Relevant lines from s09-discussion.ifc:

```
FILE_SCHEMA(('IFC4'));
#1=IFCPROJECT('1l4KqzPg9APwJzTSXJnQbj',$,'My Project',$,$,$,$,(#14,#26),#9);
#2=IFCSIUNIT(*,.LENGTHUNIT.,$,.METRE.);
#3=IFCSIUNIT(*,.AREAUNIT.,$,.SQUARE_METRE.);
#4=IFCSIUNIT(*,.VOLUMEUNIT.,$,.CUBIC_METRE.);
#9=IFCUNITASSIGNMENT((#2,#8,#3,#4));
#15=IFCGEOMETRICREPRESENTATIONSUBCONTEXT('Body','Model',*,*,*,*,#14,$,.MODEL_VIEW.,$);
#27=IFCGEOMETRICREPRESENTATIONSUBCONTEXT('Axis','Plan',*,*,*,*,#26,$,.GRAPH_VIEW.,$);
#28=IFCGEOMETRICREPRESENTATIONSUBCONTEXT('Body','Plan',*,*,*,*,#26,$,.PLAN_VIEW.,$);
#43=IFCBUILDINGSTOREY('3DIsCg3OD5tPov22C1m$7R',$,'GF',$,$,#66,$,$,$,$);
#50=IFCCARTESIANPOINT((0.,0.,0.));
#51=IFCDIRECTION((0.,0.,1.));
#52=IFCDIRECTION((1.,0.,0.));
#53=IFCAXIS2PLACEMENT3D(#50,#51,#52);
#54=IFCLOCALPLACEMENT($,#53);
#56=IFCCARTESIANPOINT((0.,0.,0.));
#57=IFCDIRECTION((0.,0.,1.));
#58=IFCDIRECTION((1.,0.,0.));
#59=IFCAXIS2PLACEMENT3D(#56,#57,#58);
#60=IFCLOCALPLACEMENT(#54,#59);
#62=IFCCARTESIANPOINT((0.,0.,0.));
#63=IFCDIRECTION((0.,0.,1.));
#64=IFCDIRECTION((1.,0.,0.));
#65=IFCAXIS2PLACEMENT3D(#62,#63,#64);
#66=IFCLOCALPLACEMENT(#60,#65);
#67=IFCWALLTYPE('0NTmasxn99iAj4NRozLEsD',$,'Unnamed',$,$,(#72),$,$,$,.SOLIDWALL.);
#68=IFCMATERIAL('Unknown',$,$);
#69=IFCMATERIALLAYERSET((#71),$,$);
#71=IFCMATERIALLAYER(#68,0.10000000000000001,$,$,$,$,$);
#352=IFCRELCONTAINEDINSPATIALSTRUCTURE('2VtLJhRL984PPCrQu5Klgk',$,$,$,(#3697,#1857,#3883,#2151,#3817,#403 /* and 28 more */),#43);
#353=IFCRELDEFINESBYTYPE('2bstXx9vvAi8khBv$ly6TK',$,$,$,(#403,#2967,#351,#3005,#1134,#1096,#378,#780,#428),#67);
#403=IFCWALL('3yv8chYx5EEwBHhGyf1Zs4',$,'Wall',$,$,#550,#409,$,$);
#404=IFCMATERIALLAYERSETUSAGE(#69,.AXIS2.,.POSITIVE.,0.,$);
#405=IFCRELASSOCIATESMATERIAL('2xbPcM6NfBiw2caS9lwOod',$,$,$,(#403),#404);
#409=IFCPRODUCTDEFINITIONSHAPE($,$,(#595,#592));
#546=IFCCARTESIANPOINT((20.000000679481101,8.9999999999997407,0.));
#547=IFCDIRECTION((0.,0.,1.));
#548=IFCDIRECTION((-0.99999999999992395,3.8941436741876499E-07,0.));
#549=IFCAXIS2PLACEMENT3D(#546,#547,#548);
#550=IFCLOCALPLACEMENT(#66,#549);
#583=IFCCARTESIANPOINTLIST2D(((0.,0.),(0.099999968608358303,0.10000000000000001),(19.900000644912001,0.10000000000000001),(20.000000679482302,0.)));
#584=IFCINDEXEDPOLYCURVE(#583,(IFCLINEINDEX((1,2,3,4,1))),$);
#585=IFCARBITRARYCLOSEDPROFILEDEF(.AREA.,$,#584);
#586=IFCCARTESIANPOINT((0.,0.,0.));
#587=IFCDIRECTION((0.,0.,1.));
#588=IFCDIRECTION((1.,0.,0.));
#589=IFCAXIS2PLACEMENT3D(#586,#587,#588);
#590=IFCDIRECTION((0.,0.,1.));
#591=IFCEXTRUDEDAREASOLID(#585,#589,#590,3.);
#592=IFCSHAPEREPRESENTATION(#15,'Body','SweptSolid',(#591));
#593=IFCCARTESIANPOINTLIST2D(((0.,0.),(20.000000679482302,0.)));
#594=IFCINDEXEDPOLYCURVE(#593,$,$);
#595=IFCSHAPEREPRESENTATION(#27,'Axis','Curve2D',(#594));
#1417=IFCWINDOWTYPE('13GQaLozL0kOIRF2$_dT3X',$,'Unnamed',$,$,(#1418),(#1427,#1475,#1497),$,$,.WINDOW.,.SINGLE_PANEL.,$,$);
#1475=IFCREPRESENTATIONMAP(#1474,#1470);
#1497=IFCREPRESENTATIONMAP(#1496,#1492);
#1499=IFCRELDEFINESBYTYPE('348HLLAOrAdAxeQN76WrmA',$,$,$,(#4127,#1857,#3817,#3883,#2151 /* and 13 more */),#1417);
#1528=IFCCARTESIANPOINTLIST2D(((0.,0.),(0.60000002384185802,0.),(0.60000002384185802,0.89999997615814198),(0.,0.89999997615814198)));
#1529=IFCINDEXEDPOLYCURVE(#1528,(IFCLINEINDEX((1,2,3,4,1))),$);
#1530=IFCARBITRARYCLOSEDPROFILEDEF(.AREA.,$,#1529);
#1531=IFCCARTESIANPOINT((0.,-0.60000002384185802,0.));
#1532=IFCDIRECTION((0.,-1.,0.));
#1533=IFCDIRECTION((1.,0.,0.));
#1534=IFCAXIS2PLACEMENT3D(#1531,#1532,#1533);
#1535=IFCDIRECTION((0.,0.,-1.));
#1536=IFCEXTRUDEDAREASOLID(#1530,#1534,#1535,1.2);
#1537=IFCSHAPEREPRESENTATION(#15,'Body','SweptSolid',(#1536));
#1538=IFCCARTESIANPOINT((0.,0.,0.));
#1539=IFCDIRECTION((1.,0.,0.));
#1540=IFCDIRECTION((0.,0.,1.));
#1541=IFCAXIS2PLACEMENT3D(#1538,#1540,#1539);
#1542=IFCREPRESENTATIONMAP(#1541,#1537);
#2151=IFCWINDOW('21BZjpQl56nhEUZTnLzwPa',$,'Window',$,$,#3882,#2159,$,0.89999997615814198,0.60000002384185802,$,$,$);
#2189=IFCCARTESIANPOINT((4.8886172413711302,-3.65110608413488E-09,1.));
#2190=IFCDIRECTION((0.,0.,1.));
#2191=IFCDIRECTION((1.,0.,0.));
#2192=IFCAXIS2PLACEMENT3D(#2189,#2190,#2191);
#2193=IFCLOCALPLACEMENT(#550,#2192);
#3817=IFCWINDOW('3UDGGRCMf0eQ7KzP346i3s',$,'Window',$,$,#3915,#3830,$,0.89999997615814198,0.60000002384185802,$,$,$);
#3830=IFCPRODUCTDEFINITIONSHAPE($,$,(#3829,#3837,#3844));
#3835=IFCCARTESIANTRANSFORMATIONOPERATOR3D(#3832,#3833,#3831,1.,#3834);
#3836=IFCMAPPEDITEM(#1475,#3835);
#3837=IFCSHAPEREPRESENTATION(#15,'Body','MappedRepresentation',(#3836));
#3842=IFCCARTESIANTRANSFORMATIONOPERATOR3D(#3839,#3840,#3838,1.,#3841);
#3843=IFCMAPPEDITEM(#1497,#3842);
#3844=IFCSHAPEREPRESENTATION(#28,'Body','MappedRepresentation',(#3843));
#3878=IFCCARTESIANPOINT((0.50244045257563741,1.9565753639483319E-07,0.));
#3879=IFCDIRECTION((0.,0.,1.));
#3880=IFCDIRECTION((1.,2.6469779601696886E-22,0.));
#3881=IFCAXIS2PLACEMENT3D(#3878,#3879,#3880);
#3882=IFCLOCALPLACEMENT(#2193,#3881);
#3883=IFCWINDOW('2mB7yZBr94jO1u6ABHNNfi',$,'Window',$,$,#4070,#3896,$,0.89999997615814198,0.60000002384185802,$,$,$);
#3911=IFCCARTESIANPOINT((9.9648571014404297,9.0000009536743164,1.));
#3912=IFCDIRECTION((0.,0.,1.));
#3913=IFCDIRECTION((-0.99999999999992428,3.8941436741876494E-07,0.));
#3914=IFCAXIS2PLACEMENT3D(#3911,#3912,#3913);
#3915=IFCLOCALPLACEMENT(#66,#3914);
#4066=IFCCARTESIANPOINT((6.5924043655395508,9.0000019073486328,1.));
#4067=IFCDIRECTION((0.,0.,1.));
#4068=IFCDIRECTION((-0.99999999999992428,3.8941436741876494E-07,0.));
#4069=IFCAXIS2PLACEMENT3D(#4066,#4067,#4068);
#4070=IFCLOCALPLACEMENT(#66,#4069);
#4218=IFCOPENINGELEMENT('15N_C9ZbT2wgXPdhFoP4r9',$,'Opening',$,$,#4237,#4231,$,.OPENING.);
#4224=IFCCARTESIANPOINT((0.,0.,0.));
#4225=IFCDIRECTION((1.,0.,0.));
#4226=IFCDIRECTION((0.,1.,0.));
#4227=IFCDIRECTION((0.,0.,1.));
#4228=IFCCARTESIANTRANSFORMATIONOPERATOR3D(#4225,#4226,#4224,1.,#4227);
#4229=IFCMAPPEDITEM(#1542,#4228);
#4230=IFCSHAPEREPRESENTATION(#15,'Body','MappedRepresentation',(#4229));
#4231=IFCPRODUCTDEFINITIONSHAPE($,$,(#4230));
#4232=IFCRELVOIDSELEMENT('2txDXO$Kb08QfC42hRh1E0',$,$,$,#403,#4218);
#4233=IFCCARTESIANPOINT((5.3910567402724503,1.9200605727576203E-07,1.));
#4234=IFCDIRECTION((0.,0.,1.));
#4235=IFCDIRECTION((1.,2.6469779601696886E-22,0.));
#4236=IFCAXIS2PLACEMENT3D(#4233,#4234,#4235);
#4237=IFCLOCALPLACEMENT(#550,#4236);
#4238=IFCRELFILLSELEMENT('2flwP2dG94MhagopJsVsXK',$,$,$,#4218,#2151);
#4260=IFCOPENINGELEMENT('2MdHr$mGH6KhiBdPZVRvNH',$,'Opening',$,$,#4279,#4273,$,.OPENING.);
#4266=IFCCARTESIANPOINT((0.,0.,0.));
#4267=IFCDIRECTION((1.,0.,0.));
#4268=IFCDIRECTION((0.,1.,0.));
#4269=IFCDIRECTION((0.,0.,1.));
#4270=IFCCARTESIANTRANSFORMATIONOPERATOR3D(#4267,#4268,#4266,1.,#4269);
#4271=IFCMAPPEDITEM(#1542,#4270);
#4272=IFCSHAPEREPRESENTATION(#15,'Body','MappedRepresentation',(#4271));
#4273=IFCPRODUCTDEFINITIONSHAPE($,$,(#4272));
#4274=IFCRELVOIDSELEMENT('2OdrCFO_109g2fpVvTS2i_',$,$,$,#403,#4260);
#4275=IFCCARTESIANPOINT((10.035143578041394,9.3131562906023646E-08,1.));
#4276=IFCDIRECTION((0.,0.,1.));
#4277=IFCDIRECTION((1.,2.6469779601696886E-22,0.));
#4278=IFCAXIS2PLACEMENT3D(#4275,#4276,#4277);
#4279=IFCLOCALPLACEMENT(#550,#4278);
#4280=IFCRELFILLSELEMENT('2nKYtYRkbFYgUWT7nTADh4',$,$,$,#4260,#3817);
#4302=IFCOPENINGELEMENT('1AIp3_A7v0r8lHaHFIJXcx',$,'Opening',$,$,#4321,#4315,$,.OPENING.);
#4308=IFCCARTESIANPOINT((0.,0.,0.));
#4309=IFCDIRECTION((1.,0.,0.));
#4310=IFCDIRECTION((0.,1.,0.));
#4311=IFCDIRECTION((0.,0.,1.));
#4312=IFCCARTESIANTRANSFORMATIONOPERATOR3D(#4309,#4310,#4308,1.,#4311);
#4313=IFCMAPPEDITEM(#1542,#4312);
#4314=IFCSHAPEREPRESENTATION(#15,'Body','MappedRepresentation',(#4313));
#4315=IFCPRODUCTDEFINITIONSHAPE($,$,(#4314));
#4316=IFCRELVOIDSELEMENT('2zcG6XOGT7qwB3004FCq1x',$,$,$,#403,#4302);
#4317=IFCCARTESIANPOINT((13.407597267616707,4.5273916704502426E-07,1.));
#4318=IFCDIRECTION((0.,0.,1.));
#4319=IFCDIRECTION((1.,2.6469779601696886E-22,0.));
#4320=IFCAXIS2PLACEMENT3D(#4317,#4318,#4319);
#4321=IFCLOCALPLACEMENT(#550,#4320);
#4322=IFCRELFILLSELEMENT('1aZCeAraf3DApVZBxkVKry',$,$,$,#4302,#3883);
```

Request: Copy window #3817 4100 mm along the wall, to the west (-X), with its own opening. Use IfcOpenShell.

```python
import ifcopenshell
import ifcopenshell.api.feature
import ifcopenshell.api.geometry
import ifcopenshell.api.root
import ifcopenshell.geom
import ifcopenshell.util.element
import ifcopenshell.util.placement
import ifcopenshell.util.shape
import ifcopenshell.util.unit

model = ifcopenshell.open("s09-discussion.ifc")
unit_scale = ifcopenshell.util.unit.calculate_unit_scale(model)
settings = ifcopenshell.geom.settings()


def volume(element):
    """Net volume in cubic metres, openings subtracted."""
    shape = ifcopenshell.geom.create_shape(settings, element)
    return ifcopenshell.util.shape.get_volume(shape.geometry)


window = model.by_guid("3UDGGRCMf0eQ7KzP346i3s")
opening = window.FillsVoids[0].RelatingOpeningElement
wall = opening.VoidsElements[0].RelatingBuildingElement
before = volume(wall)
shift = ifcopenshell.util.placement.get_local_placement(wall.ObjectPlacement)[:3, 0] * 4.1 / unit_scale

# copy_class copies the void relationship, type, container and properties, but no geometry.
new_opening = ifcopenshell.api.root.copy_class(model, product=opening)
new_opening.Representation = ifcopenshell.util.element.copy_deep(
    model, opening.Representation, exclude=["IfcGeometricRepresentationContext", "IfcRepresentationMap"]
)
new_window = ifcopenshell.api.root.copy_class(model, product=window)
new_window.Representation = ifcopenshell.util.element.copy_deep(
    model, window.Representation, exclude=["IfcGeometricRepresentationContext", "IfcRepresentationMap"]
)
ifcopenshell.api.feature.add_filling(model, opening=new_opening, element=new_window)

for old, new in ((opening, new_opening), (window, new_window)):
    matrix = ifcopenshell.util.placement.get_local_placement(old.ObjectPlacement)
    matrix[:3, 3] += shift
    ifcopenshell.api.geometry.edit_object_placement(model, product=new, matrix=matrix, is_si=False)

after = volume(wall)

print(f"wall volume {before:.3f} -> {after:.3f} m3")

model.write("s09-discussion_edited.ifc")
```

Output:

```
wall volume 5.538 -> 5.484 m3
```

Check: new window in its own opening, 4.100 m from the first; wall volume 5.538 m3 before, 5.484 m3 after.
